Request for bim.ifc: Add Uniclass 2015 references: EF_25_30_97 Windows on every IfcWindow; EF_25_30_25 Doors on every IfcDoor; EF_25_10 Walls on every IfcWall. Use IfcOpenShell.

First a look at what the model holds.

```python
import ifcopenshell

model = ifcopenshell.open("bim.ifc")
print(model.schema)
print("classifications:", [c.Name for c in model.by_type("IfcClassification")])
for ifc_class in ("IfcDoor", "IfcRoof", "IfcStair", "IfcWall", "IfcWindow"):
    print(ifc_class, len(model.by_type(ifc_class)))
```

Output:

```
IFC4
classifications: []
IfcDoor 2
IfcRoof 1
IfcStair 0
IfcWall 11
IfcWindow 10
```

```python
import ifcopenshell
import ifcopenshell.api.classification

model = ifcopenshell.open("bim.ifc")

system = ifcopenshell.api.classification.add_classification(model, classification="Uniclass 2015")

codes = {
    "IfcWindow": ("EF_25_30_97", "Windows"),
    "IfcDoor": ("EF_25_30_25", "Doors"),
    "IfcWall": ("EF_25_10", "Walls"),
}
for ifc_class, (code, name) in codes.items():
    products = model.by_type(ifc_class)
    ifcopenshell.api.classification.add_reference(
        model, products=products, classification=system, identification=code, name=name
    )
    print(code, len(products))

model.write("bim_edited.ifc")
```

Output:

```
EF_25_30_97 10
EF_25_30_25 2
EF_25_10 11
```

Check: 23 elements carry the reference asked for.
